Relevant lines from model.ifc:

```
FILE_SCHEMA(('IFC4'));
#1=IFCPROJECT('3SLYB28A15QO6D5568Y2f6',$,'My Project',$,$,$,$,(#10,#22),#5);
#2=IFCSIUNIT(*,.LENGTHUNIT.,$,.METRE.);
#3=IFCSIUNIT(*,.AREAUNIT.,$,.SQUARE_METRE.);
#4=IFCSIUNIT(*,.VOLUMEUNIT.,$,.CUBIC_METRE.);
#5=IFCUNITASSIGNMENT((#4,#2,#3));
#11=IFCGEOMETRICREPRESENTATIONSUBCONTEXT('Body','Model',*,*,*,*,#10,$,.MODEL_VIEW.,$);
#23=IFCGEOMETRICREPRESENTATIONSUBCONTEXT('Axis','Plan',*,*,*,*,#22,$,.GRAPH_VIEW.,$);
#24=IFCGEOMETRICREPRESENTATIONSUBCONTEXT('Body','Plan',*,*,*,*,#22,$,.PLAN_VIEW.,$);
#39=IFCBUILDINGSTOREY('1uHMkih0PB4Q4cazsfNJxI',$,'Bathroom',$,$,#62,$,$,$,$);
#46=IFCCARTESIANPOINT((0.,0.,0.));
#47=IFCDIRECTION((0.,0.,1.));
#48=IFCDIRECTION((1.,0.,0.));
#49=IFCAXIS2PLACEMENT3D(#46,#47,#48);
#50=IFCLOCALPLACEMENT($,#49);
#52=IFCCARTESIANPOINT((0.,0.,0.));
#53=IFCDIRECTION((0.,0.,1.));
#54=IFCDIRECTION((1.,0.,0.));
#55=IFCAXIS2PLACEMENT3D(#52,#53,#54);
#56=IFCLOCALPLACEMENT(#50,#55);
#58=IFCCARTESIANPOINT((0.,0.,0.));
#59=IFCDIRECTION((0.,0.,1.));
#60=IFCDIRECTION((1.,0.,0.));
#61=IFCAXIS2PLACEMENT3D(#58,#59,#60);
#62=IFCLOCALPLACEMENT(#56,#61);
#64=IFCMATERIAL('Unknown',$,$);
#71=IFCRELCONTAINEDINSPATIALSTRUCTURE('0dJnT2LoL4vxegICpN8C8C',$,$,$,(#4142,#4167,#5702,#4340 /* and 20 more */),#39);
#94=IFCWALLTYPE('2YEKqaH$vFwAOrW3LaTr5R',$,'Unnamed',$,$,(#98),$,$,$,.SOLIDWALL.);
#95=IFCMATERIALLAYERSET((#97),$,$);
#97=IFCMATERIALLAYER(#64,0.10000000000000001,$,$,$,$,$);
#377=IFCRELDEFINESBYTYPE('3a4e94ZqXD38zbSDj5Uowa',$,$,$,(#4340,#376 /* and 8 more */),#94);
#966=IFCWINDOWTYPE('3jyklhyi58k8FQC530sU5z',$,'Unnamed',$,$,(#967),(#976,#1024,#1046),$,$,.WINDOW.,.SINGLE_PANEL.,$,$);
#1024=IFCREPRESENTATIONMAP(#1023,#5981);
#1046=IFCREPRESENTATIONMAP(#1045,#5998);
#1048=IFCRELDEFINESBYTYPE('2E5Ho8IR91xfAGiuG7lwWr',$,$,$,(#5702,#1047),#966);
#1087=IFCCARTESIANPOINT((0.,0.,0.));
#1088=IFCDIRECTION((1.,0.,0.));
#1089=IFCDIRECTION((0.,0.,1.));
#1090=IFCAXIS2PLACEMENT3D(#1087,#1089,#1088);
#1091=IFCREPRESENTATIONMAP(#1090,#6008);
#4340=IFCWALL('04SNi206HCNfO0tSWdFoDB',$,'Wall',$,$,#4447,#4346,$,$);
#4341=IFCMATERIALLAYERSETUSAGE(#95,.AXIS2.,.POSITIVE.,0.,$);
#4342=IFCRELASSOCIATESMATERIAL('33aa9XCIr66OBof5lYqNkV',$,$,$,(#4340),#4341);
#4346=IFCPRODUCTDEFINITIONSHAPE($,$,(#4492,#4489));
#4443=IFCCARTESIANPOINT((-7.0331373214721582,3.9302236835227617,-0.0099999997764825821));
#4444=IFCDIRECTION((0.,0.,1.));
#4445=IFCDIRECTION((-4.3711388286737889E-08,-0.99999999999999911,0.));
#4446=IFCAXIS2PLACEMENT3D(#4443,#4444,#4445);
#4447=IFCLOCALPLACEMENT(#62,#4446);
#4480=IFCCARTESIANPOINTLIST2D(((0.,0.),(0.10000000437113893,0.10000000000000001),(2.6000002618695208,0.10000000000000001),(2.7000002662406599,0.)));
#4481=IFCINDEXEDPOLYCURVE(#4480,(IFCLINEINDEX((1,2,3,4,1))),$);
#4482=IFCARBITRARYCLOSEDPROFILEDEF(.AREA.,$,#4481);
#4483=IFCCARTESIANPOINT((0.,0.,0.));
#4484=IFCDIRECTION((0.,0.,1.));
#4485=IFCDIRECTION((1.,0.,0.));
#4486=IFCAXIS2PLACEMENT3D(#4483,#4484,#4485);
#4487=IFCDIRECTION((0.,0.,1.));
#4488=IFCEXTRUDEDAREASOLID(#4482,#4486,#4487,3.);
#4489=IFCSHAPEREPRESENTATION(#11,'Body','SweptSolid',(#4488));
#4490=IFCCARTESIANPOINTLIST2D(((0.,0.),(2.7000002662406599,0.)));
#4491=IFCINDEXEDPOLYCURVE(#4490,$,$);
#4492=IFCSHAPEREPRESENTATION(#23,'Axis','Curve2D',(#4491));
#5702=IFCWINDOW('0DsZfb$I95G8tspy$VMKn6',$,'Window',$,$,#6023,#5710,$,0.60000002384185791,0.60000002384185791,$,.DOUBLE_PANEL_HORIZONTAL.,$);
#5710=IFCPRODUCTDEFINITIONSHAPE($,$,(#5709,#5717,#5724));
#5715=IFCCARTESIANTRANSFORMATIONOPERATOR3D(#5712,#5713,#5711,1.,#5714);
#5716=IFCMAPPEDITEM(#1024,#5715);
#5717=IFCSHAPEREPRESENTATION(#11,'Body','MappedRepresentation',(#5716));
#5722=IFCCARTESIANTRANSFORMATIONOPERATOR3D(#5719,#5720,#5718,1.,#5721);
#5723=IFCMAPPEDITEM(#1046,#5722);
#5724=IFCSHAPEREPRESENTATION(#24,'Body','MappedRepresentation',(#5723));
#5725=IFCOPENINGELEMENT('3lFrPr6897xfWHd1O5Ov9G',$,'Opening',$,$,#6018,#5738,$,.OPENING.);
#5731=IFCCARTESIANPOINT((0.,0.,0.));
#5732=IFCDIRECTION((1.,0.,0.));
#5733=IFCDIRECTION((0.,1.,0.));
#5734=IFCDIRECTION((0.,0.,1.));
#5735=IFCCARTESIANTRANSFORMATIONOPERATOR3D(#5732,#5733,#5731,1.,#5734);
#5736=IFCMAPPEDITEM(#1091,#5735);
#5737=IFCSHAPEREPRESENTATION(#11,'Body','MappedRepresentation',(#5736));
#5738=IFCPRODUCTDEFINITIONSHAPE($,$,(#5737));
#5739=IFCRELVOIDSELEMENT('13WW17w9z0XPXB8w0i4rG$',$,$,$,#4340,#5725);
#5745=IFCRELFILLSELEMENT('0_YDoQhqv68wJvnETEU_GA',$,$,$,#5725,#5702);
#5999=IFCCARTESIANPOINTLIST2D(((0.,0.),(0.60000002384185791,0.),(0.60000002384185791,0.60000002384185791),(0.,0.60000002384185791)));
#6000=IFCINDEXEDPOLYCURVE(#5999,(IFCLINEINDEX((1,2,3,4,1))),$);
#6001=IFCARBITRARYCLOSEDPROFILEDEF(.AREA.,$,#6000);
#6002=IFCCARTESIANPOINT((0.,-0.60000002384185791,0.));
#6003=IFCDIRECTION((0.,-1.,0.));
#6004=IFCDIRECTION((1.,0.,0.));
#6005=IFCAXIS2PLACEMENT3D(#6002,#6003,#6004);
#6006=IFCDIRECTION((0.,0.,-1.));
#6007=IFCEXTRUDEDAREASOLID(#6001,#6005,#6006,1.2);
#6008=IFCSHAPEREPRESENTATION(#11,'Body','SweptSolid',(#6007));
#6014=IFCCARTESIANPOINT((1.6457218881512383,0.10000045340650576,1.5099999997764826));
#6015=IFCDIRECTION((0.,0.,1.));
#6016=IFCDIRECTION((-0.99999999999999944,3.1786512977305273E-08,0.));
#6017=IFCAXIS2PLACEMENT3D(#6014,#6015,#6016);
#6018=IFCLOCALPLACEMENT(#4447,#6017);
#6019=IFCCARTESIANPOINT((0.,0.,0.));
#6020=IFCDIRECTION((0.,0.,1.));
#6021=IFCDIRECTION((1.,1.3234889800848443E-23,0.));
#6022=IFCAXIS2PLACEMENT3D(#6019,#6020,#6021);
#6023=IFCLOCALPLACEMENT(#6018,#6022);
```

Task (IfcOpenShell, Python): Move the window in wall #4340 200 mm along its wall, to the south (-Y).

```python
import ifcopenshell
import ifcopenshell.api.geometry
import ifcopenshell.util.placement
import ifcopenshell.util.unit

model = ifcopenshell.open("model.ifc")
unit_scale = ifcopenshell.util.unit.calculate_unit_scale(model)

window = model.by_guid("0DsZfb$I95G8tspy$VMKn6")
opening = window.FillsVoids[0].RelatingOpeningElement
wall = opening.VoidsElements[0].RelatingBuildingElement

wall_matrix = ifcopenshell.util.placement.get_local_placement(wall.ObjectPlacement)
shift = wall_matrix[:3, 0] * 0.2 / unit_scale
before = ifcopenshell.util.placement.get_local_placement(window.ObjectPlacement)[:3, 3].copy()

# The window is placed relative to its opening, so it follows when the opening moves.
matrix = ifcopenshell.util.placement.get_local_placement(opening.ObjectPlacement)
matrix[:3, 3] += shift
ifcopenshell.api.geometry.edit_object_placement(
    model, product=opening, matrix=matrix, is_si=False, should_transform_children=True
)

after = ifcopenshell.util.placement.get_local_placement(window.ObjectPlacement)[:3, 3]
print("window moved by", (after - before).round(3) + 0.0)

model.write("model_v2.ifc")
```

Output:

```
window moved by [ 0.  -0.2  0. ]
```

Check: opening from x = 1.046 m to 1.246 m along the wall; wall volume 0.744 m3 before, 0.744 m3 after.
